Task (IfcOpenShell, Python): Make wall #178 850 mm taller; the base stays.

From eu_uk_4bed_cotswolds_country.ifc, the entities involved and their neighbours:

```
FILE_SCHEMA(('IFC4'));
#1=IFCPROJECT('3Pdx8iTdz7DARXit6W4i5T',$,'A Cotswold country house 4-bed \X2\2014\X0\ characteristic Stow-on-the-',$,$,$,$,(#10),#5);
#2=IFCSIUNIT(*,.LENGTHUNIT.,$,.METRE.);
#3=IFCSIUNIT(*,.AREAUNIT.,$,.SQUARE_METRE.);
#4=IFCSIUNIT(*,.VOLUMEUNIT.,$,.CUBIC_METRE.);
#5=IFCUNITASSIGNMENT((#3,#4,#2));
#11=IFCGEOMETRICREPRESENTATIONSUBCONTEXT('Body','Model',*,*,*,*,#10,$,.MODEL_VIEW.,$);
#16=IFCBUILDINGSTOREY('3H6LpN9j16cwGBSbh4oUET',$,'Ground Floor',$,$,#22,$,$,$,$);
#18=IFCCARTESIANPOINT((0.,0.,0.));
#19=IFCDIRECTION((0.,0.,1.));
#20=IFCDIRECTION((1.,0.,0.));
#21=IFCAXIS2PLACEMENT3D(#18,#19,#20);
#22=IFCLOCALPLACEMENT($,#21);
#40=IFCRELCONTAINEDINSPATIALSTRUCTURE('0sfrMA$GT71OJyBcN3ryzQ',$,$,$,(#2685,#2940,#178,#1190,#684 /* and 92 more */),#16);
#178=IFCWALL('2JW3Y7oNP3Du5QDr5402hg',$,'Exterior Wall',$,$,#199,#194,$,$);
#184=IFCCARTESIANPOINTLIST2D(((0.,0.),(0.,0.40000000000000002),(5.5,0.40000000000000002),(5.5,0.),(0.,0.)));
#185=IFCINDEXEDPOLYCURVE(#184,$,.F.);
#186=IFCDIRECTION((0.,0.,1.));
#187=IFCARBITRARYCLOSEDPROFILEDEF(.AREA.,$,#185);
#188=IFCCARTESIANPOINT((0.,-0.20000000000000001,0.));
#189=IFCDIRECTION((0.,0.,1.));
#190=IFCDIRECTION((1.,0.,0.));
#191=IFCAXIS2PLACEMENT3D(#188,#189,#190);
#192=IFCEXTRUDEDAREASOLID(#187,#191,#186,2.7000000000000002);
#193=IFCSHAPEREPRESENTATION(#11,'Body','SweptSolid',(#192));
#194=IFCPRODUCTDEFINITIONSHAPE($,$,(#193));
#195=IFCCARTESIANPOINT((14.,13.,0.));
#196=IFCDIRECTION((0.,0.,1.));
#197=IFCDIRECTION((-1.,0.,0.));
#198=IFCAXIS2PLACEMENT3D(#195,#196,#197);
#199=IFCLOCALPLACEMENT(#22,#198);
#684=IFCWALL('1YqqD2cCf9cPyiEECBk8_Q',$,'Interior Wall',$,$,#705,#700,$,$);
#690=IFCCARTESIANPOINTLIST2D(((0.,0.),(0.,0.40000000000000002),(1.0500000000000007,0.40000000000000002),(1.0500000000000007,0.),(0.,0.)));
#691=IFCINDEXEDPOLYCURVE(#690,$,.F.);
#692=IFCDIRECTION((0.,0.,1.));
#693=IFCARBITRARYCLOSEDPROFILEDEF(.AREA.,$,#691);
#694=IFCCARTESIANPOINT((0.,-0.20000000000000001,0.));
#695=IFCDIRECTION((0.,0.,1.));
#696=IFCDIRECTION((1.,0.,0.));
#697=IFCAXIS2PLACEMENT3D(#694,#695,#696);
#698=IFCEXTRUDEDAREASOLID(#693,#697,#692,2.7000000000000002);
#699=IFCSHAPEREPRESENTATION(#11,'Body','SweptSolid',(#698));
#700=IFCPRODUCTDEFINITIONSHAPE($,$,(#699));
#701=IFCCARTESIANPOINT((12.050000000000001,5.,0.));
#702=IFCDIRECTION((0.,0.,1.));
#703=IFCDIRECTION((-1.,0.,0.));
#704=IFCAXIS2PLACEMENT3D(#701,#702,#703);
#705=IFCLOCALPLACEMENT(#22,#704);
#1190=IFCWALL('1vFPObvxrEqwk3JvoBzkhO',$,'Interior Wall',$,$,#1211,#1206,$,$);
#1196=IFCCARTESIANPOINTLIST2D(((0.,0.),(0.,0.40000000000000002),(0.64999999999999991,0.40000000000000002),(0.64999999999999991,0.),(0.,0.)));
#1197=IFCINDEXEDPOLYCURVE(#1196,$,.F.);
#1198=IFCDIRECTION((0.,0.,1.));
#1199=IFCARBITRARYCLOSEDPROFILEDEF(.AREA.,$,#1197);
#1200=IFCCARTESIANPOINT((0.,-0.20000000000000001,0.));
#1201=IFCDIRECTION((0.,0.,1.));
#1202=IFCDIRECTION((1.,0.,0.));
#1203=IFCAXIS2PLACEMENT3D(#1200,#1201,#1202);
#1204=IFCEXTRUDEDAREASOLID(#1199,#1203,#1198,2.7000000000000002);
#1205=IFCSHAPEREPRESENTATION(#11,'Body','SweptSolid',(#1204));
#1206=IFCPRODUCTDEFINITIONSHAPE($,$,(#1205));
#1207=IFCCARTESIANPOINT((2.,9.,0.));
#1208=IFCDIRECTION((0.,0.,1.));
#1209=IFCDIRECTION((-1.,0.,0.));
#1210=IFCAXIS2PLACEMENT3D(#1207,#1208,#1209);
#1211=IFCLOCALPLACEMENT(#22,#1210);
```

```python
import ifcopenshell
import ifcopenshell.geom
import ifcopenshell.util.representation
import ifcopenshell.util.shape
import ifcopenshell.util.unit

model = ifcopenshell.open("eu_uk_4bed_cotswolds_country.ifc")
unit_scale = ifcopenshell.util.unit.calculate_unit_scale(model)
settings = ifcopenshell.geom.settings()


def volume(element):
    """Net volume in cubic metres, openings subtracted."""
    shape = ifcopenshell.geom.create_shape(settings, element)
    return ifcopenshell.util.shape.get_volume(shape.geometry)


wall = model.by_guid("2JW3Y7oNP3Du5QDr5402hg")
before = volume(wall)

body = ifcopenshell.util.representation.get_representation(wall, "Model", "Body")
solid = body.Items[0]
old_height = solid.Depth
solid.Depth += 0.85 / unit_scale
after = volume(wall)

print(f"height {old_height:g} -> {solid.Depth:g}, volume {before:.3f} -> {after:.3f} m3")

model.write("eu_uk_4bed_cotswolds_country_updated.ifc")
```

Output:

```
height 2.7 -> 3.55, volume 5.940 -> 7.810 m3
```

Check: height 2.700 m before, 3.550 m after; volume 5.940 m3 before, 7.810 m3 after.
